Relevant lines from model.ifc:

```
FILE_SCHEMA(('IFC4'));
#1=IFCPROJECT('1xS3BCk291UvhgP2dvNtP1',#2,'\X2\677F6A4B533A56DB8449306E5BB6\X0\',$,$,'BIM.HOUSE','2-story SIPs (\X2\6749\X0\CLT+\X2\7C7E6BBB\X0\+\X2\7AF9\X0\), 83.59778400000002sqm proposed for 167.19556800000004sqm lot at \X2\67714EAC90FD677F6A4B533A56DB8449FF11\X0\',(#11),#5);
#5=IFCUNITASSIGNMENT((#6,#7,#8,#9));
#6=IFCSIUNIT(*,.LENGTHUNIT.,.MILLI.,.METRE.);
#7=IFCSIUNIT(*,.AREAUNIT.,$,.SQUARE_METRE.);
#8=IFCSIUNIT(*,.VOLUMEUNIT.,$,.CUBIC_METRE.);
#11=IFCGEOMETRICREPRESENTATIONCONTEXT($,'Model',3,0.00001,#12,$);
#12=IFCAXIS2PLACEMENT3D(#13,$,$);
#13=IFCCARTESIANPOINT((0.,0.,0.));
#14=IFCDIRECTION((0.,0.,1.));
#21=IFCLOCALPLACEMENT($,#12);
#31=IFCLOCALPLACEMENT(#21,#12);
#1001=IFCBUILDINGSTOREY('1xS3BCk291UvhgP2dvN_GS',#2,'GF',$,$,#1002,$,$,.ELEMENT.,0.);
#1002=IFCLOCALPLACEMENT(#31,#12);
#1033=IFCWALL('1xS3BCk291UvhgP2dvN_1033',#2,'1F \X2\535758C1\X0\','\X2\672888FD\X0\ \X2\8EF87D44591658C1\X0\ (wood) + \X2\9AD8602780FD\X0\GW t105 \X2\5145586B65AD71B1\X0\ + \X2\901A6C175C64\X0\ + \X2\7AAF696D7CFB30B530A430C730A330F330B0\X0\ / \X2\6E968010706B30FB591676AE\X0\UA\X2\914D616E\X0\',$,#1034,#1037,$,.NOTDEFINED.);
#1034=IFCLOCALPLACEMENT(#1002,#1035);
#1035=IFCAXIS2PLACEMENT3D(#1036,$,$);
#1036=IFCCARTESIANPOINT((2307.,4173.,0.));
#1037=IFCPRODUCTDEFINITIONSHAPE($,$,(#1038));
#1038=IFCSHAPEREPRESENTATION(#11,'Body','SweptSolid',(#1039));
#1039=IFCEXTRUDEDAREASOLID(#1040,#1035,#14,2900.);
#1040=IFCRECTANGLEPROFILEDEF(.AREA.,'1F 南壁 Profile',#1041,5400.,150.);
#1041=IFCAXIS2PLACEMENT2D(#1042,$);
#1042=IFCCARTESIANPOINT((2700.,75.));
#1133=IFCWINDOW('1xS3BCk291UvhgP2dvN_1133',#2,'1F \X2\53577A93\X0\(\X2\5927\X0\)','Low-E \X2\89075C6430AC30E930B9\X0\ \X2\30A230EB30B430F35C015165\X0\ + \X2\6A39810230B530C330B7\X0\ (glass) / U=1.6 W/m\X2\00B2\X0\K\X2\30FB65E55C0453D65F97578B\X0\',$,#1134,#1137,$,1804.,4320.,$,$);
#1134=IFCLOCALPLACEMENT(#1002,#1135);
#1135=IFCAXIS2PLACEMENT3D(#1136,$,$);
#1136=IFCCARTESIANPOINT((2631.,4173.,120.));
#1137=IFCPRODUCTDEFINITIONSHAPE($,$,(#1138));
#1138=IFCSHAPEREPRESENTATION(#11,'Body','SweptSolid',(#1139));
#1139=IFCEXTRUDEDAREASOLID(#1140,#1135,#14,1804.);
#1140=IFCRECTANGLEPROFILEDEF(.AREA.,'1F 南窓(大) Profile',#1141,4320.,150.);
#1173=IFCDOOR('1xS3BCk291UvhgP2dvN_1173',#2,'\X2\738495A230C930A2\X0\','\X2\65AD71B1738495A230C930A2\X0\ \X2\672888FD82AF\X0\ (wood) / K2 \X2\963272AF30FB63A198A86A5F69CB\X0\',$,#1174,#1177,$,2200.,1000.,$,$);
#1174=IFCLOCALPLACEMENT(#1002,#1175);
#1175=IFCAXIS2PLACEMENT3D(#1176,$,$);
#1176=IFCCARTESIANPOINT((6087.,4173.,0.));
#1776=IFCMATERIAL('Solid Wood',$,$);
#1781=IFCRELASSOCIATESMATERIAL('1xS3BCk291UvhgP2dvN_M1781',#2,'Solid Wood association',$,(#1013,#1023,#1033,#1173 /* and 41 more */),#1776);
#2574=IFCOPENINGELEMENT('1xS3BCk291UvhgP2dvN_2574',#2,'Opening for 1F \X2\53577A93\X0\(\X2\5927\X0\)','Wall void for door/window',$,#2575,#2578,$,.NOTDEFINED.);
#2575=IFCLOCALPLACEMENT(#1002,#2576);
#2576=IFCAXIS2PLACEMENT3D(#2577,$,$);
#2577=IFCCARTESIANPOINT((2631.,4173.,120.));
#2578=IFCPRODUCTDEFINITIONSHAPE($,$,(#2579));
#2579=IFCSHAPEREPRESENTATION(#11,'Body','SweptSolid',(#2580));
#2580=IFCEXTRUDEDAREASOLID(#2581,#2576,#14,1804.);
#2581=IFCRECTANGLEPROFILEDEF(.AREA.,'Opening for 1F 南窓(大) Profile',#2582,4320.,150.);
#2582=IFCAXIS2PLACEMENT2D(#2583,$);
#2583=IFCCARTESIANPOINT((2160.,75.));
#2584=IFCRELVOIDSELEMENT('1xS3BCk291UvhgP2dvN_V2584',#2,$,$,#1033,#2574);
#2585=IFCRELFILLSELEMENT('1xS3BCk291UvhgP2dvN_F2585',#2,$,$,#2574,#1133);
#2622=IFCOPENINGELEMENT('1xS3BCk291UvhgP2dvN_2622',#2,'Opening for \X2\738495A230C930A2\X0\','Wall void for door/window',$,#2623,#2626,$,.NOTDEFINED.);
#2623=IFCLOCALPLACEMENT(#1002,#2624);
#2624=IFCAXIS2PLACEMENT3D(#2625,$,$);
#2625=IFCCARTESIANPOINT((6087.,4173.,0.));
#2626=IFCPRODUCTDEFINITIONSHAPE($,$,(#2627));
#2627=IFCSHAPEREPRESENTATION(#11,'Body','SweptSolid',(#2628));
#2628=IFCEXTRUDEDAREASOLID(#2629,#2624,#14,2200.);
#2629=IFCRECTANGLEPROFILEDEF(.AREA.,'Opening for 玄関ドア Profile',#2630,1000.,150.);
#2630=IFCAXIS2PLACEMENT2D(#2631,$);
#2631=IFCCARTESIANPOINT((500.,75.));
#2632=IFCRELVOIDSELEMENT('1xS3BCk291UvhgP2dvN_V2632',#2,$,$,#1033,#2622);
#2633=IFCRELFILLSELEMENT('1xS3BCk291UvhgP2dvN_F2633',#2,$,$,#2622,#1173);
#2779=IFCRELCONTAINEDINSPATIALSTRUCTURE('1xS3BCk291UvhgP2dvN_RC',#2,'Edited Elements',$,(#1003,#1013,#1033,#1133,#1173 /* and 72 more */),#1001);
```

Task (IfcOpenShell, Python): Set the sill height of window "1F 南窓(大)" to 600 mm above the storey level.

```python
import numpy as np
import ifcopenshell
import ifcopenshell.api.geometry
import ifcopenshell.geom
import ifcopenshell.util.element
import ifcopenshell.util.placement
import ifcopenshell.util.shape
import ifcopenshell.util.unit

model = ifcopenshell.open("model.ifc")
unit_scale = ifcopenshell.util.unit.calculate_unit_scale(model)

window = model.by_id(1133)
opening = window.FillsVoids[0].RelatingOpeningElement
storey = ifcopenshell.util.element.get_container(window, ifc_class="IfcBuildingStorey")
level = ifcopenshell.util.placement.get_local_placement(storey.ObjectPlacement)[2, 3]

# The opening's origin need not be at the sill, so measure its lowest point.
shape = ifcopenshell.geom.create_shape(ifcopenshell.geom.settings(), opening)
bottom = ifcopenshell.util.shape.get_shape_bottom_elevation(shape, shape.geometry) / unit_scale
dz = level + 0.6 / unit_scale - bottom

shift = np.array([0.0, 0.0, dz])
# The window is not placed relative to its opening, so move both.
for product in (opening, window):
    matrix = ifcopenshell.util.placement.get_local_placement(product.ObjectPlacement)
    matrix[:3, 3] += shift
    ifcopenshell.api.geometry.edit_object_placement(model, product=product, matrix=matrix, is_si=False)

print(f"moved by {dz * unit_scale:+.3f} m")

model.write("model_v2.ifc")
```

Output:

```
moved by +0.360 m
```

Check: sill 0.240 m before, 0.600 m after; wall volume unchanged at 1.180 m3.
